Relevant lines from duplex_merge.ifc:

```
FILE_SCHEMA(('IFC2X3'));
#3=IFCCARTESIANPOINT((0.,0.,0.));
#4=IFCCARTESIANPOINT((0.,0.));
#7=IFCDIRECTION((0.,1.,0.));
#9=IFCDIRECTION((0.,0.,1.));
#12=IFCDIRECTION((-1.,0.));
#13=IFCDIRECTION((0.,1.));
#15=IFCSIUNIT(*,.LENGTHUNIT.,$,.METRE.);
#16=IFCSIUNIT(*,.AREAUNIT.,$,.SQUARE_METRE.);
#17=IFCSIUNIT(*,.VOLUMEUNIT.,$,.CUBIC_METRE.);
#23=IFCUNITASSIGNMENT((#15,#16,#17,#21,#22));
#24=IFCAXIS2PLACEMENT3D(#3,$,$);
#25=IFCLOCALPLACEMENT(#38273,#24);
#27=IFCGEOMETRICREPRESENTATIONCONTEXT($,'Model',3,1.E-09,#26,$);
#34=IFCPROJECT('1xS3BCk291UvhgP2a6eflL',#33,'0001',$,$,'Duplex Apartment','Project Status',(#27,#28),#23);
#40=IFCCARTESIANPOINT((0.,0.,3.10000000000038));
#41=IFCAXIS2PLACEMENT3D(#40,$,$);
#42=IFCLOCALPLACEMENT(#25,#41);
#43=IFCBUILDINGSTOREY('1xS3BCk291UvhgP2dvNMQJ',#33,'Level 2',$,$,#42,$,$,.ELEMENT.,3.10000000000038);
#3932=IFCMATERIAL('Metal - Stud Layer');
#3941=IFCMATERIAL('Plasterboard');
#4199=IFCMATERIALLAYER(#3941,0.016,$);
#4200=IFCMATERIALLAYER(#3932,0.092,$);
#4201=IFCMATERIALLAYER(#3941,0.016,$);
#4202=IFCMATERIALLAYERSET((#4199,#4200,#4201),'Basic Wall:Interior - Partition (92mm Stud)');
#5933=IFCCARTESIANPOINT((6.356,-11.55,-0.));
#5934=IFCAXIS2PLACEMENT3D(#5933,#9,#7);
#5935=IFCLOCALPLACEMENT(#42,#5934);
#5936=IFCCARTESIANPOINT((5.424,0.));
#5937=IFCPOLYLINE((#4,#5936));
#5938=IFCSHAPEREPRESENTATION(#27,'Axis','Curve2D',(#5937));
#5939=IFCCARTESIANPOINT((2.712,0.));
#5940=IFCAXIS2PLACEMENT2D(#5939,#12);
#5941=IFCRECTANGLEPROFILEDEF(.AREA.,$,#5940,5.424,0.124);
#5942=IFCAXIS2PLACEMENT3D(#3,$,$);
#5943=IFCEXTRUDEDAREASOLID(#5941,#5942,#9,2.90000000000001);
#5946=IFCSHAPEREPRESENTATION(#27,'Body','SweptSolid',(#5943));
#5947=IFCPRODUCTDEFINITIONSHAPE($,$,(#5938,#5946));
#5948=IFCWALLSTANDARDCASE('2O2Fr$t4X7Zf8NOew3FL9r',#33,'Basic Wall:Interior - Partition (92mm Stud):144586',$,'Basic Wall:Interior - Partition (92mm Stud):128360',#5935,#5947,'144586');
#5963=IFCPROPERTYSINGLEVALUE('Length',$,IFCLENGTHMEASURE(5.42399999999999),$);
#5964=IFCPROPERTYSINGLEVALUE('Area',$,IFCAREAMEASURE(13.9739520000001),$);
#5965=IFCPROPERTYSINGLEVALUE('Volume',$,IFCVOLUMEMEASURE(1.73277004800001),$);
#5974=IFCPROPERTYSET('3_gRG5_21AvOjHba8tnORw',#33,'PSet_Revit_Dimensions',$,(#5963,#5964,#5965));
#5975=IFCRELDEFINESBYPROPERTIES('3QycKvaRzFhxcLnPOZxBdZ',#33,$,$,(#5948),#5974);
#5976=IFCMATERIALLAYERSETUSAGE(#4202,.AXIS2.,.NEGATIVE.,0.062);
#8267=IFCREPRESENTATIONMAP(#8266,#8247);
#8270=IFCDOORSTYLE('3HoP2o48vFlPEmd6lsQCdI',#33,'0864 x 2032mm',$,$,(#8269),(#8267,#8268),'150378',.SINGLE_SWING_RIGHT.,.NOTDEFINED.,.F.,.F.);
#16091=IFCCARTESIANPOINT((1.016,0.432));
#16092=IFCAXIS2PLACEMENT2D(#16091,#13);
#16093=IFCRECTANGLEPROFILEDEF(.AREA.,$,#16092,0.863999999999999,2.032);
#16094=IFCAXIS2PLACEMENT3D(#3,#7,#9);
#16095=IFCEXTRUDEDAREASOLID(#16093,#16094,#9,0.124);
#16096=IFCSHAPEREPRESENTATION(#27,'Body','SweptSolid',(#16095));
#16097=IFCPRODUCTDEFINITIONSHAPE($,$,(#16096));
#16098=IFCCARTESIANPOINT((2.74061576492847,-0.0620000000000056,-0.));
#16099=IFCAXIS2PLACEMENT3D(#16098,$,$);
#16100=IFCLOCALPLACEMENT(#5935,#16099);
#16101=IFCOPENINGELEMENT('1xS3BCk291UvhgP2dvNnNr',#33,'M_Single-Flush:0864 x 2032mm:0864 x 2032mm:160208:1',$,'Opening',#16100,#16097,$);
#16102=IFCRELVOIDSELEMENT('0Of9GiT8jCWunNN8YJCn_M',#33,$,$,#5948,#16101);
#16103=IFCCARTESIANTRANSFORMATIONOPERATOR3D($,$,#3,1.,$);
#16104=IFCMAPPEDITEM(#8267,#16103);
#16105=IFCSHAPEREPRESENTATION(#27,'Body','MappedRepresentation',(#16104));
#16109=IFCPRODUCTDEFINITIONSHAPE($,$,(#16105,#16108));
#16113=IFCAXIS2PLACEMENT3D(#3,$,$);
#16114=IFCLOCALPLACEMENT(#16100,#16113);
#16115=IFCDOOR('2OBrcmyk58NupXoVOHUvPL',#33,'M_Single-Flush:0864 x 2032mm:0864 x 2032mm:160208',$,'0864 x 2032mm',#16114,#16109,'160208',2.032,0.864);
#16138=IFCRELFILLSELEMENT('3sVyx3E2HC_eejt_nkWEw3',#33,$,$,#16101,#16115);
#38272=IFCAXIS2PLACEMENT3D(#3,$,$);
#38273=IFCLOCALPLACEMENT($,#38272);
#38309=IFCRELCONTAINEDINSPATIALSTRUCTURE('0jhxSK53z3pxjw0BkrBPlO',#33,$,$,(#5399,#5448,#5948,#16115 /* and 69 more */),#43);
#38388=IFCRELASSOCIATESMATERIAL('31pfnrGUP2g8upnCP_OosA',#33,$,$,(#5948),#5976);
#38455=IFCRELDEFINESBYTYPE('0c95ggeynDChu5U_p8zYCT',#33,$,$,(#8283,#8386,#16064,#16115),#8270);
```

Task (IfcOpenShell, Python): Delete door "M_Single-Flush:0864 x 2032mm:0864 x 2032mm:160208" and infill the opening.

```python
import ifcopenshell
import ifcopenshell.api.feature
import ifcopenshell.api.pset
import ifcopenshell.api.root
import ifcopenshell.geom
import ifcopenshell.util.element
import ifcopenshell.util.shape
import ifcopenshell.util.unit

model = ifcopenshell.open("duplex_merge.ifc")
area_scale = ifcopenshell.util.unit.calculate_unit_scale(model, "AREAUNIT")
volume_scale = ifcopenshell.util.unit.calculate_unit_scale(model, "VOLUMEUNIT")
settings = ifcopenshell.geom.settings()


def volume(element):
    """Net volume in cubic metres, openings subtracted."""
    shape = ifcopenshell.geom.create_shape(settings, element)
    return ifcopenshell.util.shape.get_volume(shape.geometry)


door = model.by_id(16115)
opening = door.FillsVoids[0].RelatingOpeningElement
wall = opening.VoidsElements[0].RelatingBuildingElement
before = volume(wall)

ifcopenshell.api.root.remove_product(model, product=door)
ifcopenshell.api.feature.remove_feature(model, feature=opening)

after = volume(wall)
thickness = 0.124  # wall thickness in metres

# Update the wall's stored quantities.
pset = model.by_id(ifcopenshell.util.element.get_pset(wall, "PSet_Revit_Dimensions", should_inherit=False)["id"])
ifcopenshell.api.pset.edit_pset(model, pset=pset, properties={
    "Area": model.create_entity("IfcAreaMeasure", after / thickness / area_scale),
    "Volume": model.create_entity("IfcVolumeMeasure", after / volume_scale),
})

print(f"wall volume {before:.3f} -> {after:.3f} m3")

model.write("duplex_merge_edited.ifc")
```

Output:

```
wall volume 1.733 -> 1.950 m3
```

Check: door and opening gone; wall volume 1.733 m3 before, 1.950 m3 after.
